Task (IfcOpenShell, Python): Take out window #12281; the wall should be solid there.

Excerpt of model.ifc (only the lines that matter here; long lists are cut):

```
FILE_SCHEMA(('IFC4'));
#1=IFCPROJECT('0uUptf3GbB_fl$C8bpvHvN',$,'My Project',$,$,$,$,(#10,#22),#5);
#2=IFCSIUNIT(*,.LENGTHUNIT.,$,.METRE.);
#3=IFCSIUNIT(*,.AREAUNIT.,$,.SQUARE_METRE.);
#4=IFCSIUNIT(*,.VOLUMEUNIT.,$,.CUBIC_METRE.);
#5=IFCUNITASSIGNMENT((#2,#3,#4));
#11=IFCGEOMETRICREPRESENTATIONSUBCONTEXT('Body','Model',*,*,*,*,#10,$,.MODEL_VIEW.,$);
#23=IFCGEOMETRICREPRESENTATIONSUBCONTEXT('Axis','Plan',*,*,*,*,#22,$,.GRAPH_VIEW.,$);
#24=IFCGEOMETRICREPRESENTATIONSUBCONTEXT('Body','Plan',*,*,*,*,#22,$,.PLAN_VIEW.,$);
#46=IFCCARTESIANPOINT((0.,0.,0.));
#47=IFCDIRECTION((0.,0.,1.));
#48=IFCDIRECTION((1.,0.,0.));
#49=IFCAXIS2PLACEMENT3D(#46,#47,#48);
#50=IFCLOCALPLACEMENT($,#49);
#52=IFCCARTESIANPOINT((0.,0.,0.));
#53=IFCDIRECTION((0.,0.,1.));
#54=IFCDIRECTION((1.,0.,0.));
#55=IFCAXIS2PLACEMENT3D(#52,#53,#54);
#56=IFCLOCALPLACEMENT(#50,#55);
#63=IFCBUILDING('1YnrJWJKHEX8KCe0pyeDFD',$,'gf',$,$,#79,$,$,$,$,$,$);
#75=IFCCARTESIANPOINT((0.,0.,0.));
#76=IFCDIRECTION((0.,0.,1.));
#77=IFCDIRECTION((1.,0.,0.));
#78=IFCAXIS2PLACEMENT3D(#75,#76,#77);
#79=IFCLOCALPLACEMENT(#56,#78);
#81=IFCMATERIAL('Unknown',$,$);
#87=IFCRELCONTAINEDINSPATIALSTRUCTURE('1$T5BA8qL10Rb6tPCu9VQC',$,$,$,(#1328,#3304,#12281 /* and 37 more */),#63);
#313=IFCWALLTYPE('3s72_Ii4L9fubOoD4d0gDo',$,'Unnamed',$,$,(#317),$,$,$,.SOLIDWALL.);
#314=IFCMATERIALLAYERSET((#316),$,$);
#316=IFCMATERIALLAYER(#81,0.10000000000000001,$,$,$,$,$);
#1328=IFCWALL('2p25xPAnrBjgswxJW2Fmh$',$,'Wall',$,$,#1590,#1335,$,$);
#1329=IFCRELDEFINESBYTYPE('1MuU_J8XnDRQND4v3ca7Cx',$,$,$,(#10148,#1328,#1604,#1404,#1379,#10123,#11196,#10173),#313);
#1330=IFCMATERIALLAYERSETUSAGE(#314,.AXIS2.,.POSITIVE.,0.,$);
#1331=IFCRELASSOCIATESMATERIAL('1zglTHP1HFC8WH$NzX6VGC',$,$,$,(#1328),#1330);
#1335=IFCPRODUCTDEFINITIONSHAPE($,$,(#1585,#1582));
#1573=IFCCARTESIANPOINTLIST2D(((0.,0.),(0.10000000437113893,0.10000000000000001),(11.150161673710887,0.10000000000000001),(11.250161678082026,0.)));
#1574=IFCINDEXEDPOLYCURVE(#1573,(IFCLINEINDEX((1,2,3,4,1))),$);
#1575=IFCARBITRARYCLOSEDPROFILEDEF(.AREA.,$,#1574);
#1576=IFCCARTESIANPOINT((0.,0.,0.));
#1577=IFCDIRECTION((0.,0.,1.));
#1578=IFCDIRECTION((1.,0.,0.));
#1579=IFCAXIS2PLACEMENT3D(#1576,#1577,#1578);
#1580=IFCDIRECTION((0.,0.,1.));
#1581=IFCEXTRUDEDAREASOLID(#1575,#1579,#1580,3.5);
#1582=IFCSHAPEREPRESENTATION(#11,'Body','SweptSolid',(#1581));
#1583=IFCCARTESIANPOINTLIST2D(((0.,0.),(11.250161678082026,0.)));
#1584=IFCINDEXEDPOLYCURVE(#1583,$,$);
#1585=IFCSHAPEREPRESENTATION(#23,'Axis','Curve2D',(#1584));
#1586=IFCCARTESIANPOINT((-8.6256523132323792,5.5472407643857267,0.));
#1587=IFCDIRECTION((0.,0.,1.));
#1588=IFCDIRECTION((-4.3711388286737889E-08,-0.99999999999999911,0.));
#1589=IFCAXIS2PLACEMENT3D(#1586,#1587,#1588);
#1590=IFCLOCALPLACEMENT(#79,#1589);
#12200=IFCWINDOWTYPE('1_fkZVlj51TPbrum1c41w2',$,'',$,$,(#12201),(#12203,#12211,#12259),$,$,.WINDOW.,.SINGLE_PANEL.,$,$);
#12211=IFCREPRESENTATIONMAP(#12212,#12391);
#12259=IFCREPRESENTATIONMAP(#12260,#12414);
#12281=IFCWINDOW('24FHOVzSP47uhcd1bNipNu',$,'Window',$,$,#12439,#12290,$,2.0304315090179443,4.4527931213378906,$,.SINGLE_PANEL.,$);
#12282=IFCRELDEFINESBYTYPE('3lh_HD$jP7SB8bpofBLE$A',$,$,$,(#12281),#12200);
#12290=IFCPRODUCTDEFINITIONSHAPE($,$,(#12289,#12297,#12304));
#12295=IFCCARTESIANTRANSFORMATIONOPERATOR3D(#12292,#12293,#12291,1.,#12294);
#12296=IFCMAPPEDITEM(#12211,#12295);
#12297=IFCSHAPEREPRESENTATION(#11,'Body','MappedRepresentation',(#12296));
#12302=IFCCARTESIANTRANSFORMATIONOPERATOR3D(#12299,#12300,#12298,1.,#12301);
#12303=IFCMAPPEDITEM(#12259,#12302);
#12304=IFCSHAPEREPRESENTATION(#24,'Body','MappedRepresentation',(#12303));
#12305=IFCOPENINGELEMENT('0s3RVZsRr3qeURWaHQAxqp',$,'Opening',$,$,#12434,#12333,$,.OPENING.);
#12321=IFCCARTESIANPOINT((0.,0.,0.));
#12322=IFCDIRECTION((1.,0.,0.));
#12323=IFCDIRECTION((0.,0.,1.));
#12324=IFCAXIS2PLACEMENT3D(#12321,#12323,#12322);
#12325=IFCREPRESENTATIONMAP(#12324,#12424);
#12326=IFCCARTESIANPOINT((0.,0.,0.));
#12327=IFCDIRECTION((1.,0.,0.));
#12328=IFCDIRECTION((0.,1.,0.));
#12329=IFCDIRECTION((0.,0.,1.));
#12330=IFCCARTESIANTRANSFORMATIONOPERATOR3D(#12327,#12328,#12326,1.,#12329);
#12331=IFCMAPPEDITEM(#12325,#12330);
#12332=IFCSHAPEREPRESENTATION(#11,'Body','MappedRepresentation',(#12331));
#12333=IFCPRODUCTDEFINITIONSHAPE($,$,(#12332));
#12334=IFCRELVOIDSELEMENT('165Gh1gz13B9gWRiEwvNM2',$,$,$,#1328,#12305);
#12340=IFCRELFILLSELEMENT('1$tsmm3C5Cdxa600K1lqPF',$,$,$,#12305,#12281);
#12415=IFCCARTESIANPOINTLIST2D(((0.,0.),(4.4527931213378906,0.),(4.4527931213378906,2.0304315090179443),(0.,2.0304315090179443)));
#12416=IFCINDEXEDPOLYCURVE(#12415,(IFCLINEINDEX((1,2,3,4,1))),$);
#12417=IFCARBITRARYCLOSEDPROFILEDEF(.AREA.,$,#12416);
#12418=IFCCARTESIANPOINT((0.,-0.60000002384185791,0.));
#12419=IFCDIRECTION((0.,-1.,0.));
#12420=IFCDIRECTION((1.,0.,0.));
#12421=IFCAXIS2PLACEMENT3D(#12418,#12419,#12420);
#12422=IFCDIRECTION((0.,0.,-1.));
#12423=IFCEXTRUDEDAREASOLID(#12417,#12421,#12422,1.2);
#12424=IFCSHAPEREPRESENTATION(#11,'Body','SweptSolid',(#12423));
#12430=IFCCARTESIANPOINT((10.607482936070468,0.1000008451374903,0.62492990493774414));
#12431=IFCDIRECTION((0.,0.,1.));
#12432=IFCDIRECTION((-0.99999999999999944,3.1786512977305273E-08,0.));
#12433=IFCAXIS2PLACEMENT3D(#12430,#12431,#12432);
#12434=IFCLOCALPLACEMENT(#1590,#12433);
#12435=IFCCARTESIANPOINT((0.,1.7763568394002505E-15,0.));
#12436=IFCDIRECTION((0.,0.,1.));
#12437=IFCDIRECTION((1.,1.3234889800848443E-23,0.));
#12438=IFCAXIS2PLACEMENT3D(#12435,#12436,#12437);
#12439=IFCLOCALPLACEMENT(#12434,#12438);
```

```python
import ifcopenshell
import ifcopenshell.api.feature
import ifcopenshell.api.root
import ifcopenshell.geom
import ifcopenshell.util.shape

model = ifcopenshell.open("model.ifc")
settings = ifcopenshell.geom.settings()


def volume(element):
    """Net volume in cubic metres, openings subtracted."""
    shape = ifcopenshell.geom.create_shape(settings, element)
    return ifcopenshell.util.shape.get_volume(shape.geometry)


window = model.by_guid("24FHOVzSP47uhcd1bNipNu")
opening = window.FillsVoids[0].RelatingOpeningElement
wall = opening.VoidsElements[0].RelatingBuildingElement
before = volume(wall)

ifcopenshell.api.root.remove_product(model, product=window)
ifcopenshell.api.feature.remove_feature(model, feature=opening)

after = volume(wall)

print(f"wall volume {before:.3f} -> {after:.3f} m3")

model.write("model_edited.ifc")
```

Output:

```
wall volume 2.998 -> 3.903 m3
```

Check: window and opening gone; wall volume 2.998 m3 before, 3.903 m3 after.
